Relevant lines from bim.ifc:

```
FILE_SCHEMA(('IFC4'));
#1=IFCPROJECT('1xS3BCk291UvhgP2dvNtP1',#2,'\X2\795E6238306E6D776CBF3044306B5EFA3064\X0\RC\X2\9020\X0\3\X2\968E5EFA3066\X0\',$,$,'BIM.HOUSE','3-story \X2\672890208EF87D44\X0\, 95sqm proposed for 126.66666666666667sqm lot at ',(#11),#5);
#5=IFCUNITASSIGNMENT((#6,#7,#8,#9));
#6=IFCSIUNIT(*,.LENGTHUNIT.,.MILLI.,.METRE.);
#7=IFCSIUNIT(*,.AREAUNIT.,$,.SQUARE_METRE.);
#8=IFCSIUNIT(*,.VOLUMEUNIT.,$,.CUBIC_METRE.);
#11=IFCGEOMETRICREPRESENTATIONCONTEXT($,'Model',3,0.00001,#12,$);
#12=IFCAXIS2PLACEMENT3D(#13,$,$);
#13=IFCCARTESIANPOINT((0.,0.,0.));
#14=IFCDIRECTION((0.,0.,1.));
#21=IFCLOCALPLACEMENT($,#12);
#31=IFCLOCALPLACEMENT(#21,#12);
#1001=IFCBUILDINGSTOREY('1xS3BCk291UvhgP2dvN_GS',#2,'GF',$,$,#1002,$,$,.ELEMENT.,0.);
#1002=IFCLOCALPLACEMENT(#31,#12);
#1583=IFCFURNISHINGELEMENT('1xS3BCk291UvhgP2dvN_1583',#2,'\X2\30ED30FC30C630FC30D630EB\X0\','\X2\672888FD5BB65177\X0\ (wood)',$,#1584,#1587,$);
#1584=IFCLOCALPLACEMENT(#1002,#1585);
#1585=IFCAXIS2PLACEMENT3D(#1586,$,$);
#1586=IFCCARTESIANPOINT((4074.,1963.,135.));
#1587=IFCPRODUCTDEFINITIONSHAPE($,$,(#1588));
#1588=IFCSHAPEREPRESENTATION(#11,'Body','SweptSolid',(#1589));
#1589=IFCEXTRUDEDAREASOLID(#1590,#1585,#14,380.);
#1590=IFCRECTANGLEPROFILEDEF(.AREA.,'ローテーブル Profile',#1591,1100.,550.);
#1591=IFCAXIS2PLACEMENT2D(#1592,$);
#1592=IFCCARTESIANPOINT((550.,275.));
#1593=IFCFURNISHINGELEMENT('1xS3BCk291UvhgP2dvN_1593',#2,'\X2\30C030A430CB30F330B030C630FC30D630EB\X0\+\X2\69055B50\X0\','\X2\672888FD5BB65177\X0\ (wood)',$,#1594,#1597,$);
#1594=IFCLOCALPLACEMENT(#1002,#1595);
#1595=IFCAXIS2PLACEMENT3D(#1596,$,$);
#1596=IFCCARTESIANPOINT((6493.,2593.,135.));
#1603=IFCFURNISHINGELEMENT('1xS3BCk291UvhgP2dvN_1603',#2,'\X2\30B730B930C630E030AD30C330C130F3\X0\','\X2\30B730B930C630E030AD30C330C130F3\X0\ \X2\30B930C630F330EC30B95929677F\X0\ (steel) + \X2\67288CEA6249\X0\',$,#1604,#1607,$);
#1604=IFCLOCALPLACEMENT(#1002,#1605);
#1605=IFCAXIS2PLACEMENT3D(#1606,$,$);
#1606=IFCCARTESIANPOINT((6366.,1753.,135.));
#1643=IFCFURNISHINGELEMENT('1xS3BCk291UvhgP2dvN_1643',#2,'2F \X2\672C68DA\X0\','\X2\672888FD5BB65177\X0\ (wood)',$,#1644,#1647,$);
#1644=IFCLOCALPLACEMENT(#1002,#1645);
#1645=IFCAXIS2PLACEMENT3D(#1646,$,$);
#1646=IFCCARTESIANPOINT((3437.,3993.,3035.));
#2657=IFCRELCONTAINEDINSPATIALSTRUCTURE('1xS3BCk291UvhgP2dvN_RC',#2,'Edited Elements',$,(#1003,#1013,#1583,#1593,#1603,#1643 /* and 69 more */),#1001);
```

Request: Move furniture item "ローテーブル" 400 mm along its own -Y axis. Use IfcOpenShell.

```python
import ifcopenshell
import ifcopenshell.api.geometry
import ifcopenshell.util.placement

model = ifcopenshell.open("bim.ifc")

item = model.by_guid("1xS3BCk291UvhgP2dvN_1583")
matrix = ifcopenshell.util.placement.get_local_placement(item.ObjectPlacement)
matrix[:3, 3] -= matrix[:3, 1] * 400.0
ifcopenshell.api.geometry.edit_object_placement(model, product=item, matrix=matrix, is_si=False)

print(ifcopenshell.util.placement.get_local_placement(item.ObjectPlacement).round(3) + 0.0)

model.write("bim_edited.ifc")
```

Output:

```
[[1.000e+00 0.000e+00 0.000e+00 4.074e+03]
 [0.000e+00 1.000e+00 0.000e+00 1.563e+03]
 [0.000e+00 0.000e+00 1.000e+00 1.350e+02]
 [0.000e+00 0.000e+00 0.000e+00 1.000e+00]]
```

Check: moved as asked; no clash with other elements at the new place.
